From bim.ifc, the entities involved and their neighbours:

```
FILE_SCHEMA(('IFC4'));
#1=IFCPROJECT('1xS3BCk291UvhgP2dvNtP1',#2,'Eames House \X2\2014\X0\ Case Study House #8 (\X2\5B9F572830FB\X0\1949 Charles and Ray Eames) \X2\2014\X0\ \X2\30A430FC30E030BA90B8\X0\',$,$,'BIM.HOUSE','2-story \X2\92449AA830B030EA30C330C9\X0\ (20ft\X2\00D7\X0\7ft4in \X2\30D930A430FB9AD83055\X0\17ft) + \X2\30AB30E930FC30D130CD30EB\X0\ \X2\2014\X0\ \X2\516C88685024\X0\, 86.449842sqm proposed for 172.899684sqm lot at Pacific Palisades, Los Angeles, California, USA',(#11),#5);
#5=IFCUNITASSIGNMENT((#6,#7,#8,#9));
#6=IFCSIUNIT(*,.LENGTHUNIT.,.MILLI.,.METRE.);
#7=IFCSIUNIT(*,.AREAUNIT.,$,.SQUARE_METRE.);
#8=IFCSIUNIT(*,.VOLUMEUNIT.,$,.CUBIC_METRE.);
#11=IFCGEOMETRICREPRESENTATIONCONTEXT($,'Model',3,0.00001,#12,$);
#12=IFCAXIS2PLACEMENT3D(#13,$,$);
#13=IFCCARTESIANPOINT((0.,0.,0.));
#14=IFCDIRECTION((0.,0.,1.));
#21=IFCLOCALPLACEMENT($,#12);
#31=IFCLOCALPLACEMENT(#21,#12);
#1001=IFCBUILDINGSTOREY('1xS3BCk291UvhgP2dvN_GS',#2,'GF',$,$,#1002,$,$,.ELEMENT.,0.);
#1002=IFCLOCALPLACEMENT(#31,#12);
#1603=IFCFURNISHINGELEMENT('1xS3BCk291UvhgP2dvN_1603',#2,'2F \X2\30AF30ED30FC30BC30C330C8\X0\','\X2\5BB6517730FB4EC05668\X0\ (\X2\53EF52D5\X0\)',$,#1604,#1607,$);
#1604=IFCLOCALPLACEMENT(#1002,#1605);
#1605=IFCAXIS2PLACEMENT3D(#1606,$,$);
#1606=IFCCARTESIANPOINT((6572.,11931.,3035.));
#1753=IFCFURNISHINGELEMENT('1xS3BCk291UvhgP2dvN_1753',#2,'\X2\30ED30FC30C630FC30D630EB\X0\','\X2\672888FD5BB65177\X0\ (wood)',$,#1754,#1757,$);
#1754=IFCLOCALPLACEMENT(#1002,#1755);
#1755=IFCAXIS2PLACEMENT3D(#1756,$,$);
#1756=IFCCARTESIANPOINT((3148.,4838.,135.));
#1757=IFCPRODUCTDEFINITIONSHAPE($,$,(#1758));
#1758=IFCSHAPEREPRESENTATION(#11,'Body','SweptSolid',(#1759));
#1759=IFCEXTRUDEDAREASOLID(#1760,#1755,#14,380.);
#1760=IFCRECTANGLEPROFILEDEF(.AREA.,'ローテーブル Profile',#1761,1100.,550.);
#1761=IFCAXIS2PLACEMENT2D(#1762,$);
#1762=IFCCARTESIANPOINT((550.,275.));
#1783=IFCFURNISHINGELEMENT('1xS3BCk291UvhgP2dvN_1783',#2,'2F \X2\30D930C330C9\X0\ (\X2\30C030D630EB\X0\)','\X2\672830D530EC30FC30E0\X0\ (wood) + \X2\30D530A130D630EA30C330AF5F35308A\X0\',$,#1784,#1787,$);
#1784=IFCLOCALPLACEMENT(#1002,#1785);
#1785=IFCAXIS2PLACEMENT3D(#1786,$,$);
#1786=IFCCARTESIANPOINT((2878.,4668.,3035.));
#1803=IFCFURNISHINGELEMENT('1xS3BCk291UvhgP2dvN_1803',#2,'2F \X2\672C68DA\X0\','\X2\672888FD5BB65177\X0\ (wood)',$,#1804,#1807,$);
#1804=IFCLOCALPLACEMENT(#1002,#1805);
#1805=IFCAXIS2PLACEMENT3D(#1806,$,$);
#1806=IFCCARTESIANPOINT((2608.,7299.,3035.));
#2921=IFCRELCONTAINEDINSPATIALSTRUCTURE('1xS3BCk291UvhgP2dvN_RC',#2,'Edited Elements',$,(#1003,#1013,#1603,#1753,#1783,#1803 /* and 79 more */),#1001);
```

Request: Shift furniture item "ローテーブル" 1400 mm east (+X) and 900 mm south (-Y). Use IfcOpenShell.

```python
import ifcopenshell
import ifcopenshell.api.geometry
import ifcopenshell.util.placement
import ifcopenshell.util.unit

model = ifcopenshell.open("bim.ifc")
unit_scale = ifcopenshell.util.unit.calculate_unit_scale(model)

item = model.by_guid("1xS3BCk291UvhgP2dvN_1753")
matrix = ifcopenshell.util.placement.get_local_placement(item.ObjectPlacement)
matrix[0, 3] += 1.4 / unit_scale
matrix[1, 3] -= 0.9 / unit_scale
ifcopenshell.api.geometry.edit_object_placement(model, product=item, matrix=matrix, is_si=False)

print(ifcopenshell.util.placement.get_local_placement(item.ObjectPlacement).round(3) + 0.0)

model.write("bim-out.ifc")
```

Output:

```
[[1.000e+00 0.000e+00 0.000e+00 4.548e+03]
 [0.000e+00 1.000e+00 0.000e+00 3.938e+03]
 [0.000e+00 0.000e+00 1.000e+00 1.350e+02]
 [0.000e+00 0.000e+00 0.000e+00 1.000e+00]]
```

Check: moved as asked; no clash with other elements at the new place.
